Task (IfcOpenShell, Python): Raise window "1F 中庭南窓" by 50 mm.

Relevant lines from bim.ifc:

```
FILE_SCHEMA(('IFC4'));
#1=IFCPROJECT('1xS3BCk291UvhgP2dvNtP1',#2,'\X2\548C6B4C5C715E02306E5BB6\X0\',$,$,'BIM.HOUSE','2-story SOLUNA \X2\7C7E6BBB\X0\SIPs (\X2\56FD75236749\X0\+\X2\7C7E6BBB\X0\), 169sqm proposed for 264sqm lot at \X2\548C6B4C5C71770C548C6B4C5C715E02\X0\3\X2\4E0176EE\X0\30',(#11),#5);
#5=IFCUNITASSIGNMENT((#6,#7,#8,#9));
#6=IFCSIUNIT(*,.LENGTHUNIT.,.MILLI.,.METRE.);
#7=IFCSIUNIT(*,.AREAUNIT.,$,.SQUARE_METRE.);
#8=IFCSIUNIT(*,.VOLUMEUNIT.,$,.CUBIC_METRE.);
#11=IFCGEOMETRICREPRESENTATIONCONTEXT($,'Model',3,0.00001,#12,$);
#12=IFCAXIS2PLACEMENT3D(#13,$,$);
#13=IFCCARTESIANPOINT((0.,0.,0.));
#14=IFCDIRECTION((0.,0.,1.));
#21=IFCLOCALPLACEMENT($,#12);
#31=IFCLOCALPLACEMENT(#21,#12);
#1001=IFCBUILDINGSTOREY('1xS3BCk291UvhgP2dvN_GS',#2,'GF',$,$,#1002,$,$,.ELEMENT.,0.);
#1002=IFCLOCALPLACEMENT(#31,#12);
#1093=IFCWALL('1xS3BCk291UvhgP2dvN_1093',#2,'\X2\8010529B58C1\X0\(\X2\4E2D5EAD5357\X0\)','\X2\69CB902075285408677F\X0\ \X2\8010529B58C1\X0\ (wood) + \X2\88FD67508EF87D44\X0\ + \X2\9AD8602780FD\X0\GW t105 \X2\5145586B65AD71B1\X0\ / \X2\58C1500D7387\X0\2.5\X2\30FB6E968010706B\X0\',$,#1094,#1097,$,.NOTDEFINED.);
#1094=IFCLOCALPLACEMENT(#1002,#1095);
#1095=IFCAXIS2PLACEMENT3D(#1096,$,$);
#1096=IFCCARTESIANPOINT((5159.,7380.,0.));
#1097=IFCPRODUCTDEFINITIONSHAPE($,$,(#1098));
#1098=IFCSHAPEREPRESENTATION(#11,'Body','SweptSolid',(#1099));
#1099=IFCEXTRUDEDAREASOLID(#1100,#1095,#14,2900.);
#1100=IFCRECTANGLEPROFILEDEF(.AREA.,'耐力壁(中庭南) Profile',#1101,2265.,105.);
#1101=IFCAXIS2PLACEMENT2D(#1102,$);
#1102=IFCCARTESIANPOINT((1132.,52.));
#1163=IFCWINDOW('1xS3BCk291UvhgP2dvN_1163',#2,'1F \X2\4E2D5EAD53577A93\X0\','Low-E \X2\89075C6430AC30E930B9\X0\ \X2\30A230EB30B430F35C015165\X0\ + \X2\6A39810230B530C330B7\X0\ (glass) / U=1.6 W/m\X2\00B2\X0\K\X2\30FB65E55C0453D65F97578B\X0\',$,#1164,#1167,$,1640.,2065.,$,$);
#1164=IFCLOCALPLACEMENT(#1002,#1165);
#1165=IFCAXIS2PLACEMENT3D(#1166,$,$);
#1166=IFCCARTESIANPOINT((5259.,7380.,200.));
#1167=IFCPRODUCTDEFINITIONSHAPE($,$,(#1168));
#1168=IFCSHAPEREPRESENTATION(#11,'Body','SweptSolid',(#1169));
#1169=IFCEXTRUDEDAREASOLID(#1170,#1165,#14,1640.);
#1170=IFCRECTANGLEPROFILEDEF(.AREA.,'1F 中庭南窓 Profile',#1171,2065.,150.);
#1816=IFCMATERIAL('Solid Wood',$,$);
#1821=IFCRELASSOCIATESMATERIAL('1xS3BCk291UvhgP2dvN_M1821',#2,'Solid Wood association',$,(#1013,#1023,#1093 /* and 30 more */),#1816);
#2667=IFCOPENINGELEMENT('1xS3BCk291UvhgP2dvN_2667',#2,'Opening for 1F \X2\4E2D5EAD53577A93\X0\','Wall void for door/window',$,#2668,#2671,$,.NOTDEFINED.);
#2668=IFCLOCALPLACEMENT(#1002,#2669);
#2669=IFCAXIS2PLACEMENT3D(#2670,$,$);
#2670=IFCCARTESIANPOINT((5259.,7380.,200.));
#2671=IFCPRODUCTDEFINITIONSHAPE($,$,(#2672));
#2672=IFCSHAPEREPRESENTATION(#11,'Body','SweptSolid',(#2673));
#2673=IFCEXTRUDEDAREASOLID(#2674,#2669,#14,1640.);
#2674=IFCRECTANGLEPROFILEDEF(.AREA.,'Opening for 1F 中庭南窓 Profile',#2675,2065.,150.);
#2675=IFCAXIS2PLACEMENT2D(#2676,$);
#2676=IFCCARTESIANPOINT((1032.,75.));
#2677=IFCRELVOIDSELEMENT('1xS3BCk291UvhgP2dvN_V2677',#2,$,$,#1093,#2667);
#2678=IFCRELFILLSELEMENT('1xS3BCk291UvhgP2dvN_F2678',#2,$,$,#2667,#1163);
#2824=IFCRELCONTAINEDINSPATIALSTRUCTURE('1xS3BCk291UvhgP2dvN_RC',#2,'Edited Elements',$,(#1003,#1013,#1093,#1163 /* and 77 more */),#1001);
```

```python
import numpy as np
import ifcopenshell
import ifcopenshell.api.geometry
import ifcopenshell.util.placement
import ifcopenshell.util.unit

model = ifcopenshell.open("bim.ifc")
unit_scale = ifcopenshell.util.unit.calculate_unit_scale(model)

window = model.by_guid("1xS3BCk291UvhgP2dvN_1163")
opening = window.FillsVoids[0].RelatingOpeningElement
dz = 50.0

shift = np.array([0.0, 0.0, dz])
# The window is not placed relative to its opening, so move both.
for product in (opening, window):
    matrix = ifcopenshell.util.placement.get_local_placement(product.ObjectPlacement)
    matrix[:3, 3] += shift
    ifcopenshell.api.geometry.edit_object_placement(model, product=product, matrix=matrix, is_si=False)

print(f"moved by {dz * unit_scale:+.3f} m")

model.write("bim_edited.ifc")
```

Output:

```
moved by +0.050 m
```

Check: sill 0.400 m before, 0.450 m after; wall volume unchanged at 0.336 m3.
